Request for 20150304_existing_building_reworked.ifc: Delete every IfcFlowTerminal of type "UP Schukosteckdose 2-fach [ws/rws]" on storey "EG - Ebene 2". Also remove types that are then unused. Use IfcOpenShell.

First a look at what the model holds.

```python
import ifcopenshell
import ifcopenshell.util.element

model = ifcopenshell.open("20150304_existing_building_reworked.ifc")
print(model.schema)
storey = next(s for s in model.by_type("IfcBuildingStorey") if s.Name == "EG - Ebene 2")
terminals = [e for e in ifcopenshell.util.element.get_decomposition(storey) if e.is_a("IfcFlowTerminal")]
seen = {}
for e in terminals:
    element_type = ifcopenshell.util.element.get_type(e)
    name = element_type.Name if element_type not in (None, e) else None
    seen[name] = seen.get(name, 0) + 1
for name, count in sorted(seen.items(), key=str):
    print(count, "x", name)
```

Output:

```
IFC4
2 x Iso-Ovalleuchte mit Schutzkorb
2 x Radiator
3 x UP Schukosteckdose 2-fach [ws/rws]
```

```python
import ifcopenshell
import ifcopenshell.api.root
import ifcopenshell.util.element

model = ifcopenshell.open("20150304_existing_building_reworked.ifc")

storey = next(s for s in model.by_type("IfcBuildingStorey") if s.Name == "EG - Ebene 2")
terminals = [e for e in ifcopenshell.util.element.get_decomposition(storey) if e.is_a("IfcFlowTerminal")]
targets = [e for e in terminals if (t := ifcopenshell.util.element.get_type(e)) not in (None, e) and t.Name == "UP Schukosteckdose 2-fach [ws/rws]"]
types = {ifcopenshell.util.element.get_type(e) for e in targets} - {None, *targets}

for e in targets:
    ifcopenshell.api.root.remove_product(model, product=e)
print(len(targets), "removed")

unused = [t for t in types if not ifcopenshell.util.element.get_types(t)]
for t in unused:
    ifcopenshell.api.root.remove_product(model, product=t)
print(len(unused), "unused types removed")

model.write("20150304_existing_building_reworked_v2.ifc")
```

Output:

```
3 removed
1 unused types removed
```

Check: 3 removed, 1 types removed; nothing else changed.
